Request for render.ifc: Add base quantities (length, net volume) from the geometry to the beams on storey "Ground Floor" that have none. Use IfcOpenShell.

First a look at what the model holds.

```python
import ifcopenshell
import ifcopenshell.util.element
import ifcopenshell.util.unit

model = ifcopenshell.open("render.ifc")
print(model.schema)
for unit_type in ("LENGTHUNIT", "AREAUNIT", "VOLUMEUNIT"):
    print(unit_type, ifcopenshell.util.unit.calculate_unit_scale(model, unit_type))
storey = next(s for s in model.by_type("IfcBuildingStorey") if s.Name == "Ground Floor")
beams = [e for e in ifcopenshell.util.element.get_decomposition(storey) if e.is_a("IfcBeam")]
for e in sorted(beams, key=lambda e: e.id()):
    print(e.id(), e.is_a(), e.Name, list(ifcopenshell.util.element.get_psets(e, qtos_only=True)), sep=" | ")
```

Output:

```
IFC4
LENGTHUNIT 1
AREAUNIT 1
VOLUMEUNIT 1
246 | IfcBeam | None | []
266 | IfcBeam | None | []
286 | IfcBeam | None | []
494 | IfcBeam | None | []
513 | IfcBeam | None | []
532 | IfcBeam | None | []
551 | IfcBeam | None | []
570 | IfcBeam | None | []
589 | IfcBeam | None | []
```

```python
import ifcopenshell
import ifcopenshell.api.pset
import ifcopenshell.geom
import ifcopenshell.util.element
import ifcopenshell.util.shape
import ifcopenshell.util.unit

model = ifcopenshell.open("render.ifc")
unit_scale = ifcopenshell.util.unit.calculate_unit_scale(model)
volume_scale = ifcopenshell.util.unit.calculate_unit_scale(model, "VOLUMEUNIT")
settings = ifcopenshell.geom.settings()

storey = next(s for s in model.by_type("IfcBuildingStorey") if s.Name == "Ground Floor")
beams = [e for e in ifcopenshell.util.element.get_decomposition(storey) if e.is_a("IfcBeam")]

for e in sorted(beams, key=lambda e: e.id()):
    if ifcopenshell.util.element.get_psets(e, qtos_only=True, should_inherit=False):
        continue
    # Geometry comes back in metres, in the element's own axes.
    shape = ifcopenshell.geom.create_shape(settings, e)
    values = {
        "Length": ifcopenshell.util.shape.get_max_xyz(shape.geometry) / unit_scale,
        "NetVolume": ifcopenshell.util.shape.get_volume(shape.geometry) / volume_scale,
    }
    qto = ifcopenshell.api.pset.add_qto(model, product=e, name="Qto_BeamBaseQuantities")
    ifcopenshell.api.pset.edit_qto(model, qto=qto, properties=values)
    print(e.id(), {k: round(v, 3) for k, v in values.items()})

model.write("render_rev.ifc")
```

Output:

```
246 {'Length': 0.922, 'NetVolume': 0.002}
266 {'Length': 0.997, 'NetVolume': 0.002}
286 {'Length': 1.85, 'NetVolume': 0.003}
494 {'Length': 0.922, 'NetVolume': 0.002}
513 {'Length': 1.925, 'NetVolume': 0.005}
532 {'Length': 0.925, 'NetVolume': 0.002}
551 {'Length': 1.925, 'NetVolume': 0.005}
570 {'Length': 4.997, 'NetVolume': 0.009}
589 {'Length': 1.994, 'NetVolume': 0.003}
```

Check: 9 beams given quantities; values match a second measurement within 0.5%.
